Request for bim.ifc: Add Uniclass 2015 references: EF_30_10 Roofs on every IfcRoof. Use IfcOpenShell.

First a look at what the model holds.

```python
import ifcopenshell

model = ifcopenshell.open("bim.ifc")
print(model.schema)
print("classifications:", [c.Name for c in model.by_type("IfcClassification")])
for ifc_class in ("IfcDoor", "IfcRoof", "IfcStair", "IfcWall", "IfcWindow"):
    print(ifc_class, len(model.by_type(ifc_class)))
```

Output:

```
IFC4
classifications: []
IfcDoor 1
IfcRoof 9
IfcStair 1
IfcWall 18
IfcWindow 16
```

```python
import ifcopenshell
import ifcopenshell.api.classification

model = ifcopenshell.open("bim.ifc")

system = ifcopenshell.api.classification.add_classification(model, classification="Uniclass 2015")

codes = {
    "IfcRoof": ("EF_30_10", "Roofs"),
}
for ifc_class, (code, name) in codes.items():
    products = model.by_type(ifc_class)
    ifcopenshell.api.classification.add_reference(
        model, products=products, classification=system, identification=code, name=name
    )
    print(code, len(products))

model.write("bim-out.ifc")
```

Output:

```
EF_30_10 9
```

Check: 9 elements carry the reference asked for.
